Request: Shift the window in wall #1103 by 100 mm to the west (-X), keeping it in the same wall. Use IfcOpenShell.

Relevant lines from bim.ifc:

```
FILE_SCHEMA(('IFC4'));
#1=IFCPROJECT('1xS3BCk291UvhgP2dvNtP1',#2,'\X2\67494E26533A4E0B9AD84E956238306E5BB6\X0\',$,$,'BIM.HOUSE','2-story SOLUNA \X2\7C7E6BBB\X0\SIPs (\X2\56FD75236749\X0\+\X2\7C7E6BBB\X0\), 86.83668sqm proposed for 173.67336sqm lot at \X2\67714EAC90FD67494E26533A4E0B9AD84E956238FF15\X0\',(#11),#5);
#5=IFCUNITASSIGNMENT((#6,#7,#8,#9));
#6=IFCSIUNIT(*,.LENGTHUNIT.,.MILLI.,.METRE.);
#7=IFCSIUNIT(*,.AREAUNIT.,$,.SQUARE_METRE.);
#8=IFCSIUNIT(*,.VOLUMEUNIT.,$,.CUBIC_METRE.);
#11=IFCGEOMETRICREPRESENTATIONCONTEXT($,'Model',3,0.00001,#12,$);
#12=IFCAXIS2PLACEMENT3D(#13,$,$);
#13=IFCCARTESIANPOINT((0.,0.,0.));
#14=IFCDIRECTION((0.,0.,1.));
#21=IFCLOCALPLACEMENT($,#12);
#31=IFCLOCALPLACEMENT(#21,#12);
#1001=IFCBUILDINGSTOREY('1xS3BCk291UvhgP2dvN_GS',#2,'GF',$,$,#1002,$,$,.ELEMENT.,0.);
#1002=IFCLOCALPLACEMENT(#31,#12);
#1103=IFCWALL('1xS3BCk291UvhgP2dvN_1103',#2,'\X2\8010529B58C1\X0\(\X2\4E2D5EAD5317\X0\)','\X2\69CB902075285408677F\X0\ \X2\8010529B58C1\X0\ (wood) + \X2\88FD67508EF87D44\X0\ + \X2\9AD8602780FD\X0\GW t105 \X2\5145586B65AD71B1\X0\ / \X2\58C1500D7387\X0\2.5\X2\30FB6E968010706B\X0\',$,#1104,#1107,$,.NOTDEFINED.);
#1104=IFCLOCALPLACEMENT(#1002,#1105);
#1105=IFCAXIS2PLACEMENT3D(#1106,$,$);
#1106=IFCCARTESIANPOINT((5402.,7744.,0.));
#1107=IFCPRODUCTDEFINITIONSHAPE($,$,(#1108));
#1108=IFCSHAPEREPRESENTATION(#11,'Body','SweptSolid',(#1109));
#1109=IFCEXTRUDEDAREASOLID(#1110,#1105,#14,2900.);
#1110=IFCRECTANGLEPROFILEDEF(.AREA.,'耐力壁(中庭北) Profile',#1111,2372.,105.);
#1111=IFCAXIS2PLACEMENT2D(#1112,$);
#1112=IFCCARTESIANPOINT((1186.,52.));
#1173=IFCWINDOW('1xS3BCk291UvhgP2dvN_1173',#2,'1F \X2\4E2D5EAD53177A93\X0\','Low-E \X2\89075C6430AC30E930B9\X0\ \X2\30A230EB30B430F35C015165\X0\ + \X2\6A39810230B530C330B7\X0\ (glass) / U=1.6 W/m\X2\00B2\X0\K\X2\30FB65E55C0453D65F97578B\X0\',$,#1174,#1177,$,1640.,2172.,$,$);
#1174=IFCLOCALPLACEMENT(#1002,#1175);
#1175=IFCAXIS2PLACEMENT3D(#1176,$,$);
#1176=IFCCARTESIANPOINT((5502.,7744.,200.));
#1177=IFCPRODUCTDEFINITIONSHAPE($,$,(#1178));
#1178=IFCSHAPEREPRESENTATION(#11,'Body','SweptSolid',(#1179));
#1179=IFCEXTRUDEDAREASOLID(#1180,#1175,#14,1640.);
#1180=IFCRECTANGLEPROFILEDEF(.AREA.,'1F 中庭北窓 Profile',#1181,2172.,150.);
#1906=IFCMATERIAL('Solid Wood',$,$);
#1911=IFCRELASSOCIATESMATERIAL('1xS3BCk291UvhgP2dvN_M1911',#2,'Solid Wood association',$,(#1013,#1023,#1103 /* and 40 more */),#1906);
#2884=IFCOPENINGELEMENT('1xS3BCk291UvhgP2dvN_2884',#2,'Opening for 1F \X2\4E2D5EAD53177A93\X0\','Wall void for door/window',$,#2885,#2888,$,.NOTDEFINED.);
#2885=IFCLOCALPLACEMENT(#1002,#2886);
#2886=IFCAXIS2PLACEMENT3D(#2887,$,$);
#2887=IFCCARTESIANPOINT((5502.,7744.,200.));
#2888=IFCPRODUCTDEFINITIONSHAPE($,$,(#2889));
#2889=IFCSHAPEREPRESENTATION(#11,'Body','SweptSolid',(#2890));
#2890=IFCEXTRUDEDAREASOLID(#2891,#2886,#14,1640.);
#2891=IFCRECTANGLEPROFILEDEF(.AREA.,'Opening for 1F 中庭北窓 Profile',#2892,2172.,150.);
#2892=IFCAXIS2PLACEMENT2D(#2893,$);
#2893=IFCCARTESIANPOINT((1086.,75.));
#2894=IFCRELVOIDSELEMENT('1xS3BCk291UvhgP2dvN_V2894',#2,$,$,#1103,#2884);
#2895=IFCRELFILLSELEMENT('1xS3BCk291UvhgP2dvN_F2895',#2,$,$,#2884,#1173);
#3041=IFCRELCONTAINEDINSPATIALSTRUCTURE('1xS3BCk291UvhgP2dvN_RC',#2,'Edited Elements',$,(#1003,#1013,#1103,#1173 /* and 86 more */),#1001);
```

```python
import ifcopenshell
import ifcopenshell.api.geometry
import ifcopenshell.util.placement

model = ifcopenshell.open("bim.ifc")

window = model.by_guid("1xS3BCk291UvhgP2dvN_1173")
opening = window.FillsVoids[0].RelatingOpeningElement
wall = opening.VoidsElements[0].RelatingBuildingElement

wall_matrix = ifcopenshell.util.placement.get_local_placement(wall.ObjectPlacement)
shift = wall_matrix[:3, 0] * -100.0
before = ifcopenshell.util.placement.get_local_placement(window.ObjectPlacement)[:3, 3].copy()

# The window is not placed relative to its opening, so move both.
for product in (opening, window):
    matrix = ifcopenshell.util.placement.get_local_placement(product.ObjectPlacement)
    matrix[:3, 3] += shift
    ifcopenshell.api.geometry.edit_object_placement(model, product=product, matrix=matrix, is_si=False)

after = ifcopenshell.util.placement.get_local_placement(window.ObjectPlacement)[:3, 3]
print("window moved by", (after - before).round(3) + 0.0)

model.write("bim_updated.ifc")
```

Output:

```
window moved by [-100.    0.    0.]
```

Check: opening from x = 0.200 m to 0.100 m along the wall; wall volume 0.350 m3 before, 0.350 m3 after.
